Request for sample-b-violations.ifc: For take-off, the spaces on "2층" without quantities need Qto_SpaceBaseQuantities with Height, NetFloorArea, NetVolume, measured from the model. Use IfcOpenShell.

First a look at what the model holds.

```python
import ifcopenshell
import ifcopenshell.util.element
import ifcopenshell.util.unit

model = ifcopenshell.open("sample-b-violations.ifc")
print(model.schema)
for unit_type in ("LENGTHUNIT", "AREAUNIT", "VOLUMEUNIT"):
    print(unit_type, ifcopenshell.util.unit.calculate_unit_scale(model, unit_type))
storey = next(s for s in model.by_type("IfcBuildingStorey") if s.Name == "2층")
spaces = [e for e in ifcopenshell.util.element.get_decomposition(storey) if e.is_a("IfcSpace")]
for e in sorted(spaces, key=lambda e: e.id()):
    print(e.id(), e.is_a(), e.Name, list(ifcopenshell.util.element.get_psets(e, qtos_only=True)), sep=" | ")
```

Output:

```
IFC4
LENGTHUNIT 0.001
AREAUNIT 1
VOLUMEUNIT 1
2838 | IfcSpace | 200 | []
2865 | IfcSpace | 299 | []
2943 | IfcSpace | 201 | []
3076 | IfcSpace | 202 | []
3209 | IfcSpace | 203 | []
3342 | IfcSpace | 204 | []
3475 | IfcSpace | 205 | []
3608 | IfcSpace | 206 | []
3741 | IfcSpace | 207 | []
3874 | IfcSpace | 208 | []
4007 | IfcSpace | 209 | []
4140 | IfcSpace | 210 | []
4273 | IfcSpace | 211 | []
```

```python
import ifcopenshell
import ifcopenshell.api.pset
import ifcopenshell.geom
import ifcopenshell.util.element
import ifcopenshell.util.shape
import ifcopenshell.util.unit

model = ifcopenshell.open("sample-b-violations.ifc")
unit_scale = ifcopenshell.util.unit.calculate_unit_scale(model)
area_scale = ifcopenshell.util.unit.calculate_unit_scale(model, "AREAUNIT")
volume_scale = ifcopenshell.util.unit.calculate_unit_scale(model, "VOLUMEUNIT")
settings = ifcopenshell.geom.settings()

storey = next(s for s in model.by_type("IfcBuildingStorey") if s.Name == "2층")
spaces = [e for e in ifcopenshell.util.element.get_decomposition(storey) if e.is_a("IfcSpace")]

for e in sorted(spaces, key=lambda e: e.id()):
    if ifcopenshell.util.element.get_psets(e, qtos_only=True, should_inherit=False):
        continue
    # Geometry comes back in metres, in the element's own axes.
    shape = ifcopenshell.geom.create_shape(settings, e)
    values = {
        "Height": ifcopenshell.util.shape.get_z(shape.geometry) / unit_scale,
        "NetFloorArea": ifcopenshell.util.shape.get_footprint_area(shape.geometry) / area_scale,
        "NetVolume": ifcopenshell.util.shape.get_volume(shape.geometry) / volume_scale,
    }
    qto = ifcopenshell.api.pset.add_qto(model, product=e, name="Qto_SpaceBaseQuantities")
    ifcopenshell.api.pset.edit_qto(model, qto=qto, properties=values)
    print(e.id(), {k: round(v, 3) for k, v in values.items()})

model.write("sample-b-violations_edited.ifc")
```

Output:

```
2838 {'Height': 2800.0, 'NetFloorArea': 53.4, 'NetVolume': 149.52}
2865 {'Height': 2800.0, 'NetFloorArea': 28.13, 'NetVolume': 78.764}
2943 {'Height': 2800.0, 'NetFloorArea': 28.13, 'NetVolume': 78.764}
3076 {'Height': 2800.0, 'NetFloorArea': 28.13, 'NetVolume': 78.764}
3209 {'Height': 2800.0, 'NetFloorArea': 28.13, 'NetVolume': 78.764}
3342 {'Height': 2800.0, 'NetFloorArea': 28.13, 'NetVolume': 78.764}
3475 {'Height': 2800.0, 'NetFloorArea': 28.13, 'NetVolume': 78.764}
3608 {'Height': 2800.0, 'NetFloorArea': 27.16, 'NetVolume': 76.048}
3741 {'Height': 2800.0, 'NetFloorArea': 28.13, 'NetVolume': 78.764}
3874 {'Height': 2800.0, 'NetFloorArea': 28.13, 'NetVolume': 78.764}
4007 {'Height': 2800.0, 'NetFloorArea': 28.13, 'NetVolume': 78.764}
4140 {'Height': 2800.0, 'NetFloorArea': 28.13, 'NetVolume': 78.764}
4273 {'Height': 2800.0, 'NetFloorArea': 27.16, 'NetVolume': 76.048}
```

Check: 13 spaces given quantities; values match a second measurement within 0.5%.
